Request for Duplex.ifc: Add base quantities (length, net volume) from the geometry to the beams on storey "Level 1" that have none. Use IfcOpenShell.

First a look at what the model holds.

```python
import ifcopenshell
import ifcopenshell.util.element
import ifcopenshell.util.unit

model = ifcopenshell.open("Duplex.ifc")
print(model.schema)
for unit_type in ("LENGTHUNIT", "AREAUNIT", "VOLUMEUNIT"):
    print(unit_type, ifcopenshell.util.unit.calculate_unit_scale(model, unit_type))
storey = next(s for s in model.by_type("IfcBuildingStorey") if s.Name == "Level 1")
beams = [e for e in ifcopenshell.util.element.get_decomposition(storey) if e.is_a("IfcBeam")]
for e in sorted(beams, key=lambda e: e.id()):
    print(e.id(), e.is_a(), e.Name, list(ifcopenshell.util.element.get_psets(e, qtos_only=True)), sep=" | ")
```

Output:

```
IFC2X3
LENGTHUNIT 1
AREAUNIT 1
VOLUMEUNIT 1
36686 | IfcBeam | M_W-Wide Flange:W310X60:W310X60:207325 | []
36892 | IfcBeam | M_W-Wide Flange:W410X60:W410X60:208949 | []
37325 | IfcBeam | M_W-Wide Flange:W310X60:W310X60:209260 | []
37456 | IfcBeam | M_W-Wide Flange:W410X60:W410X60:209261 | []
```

```python
import ifcopenshell
import ifcopenshell.api.pset
import ifcopenshell.geom
import ifcopenshell.util.element
import ifcopenshell.util.shape
import ifcopenshell.util.unit

model = ifcopenshell.open("Duplex.ifc")
unit_scale = ifcopenshell.util.unit.calculate_unit_scale(model)
volume_scale = ifcopenshell.util.unit.calculate_unit_scale(model, "VOLUMEUNIT")
settings = ifcopenshell.geom.settings()

storey = next(s for s in model.by_type("IfcBuildingStorey") if s.Name == "Level 1")
beams = [e for e in ifcopenshell.util.element.get_decomposition(storey) if e.is_a("IfcBeam")]

for e in sorted(beams, key=lambda e: e.id()):
    if ifcopenshell.util.element.get_psets(e, qtos_only=True, should_inherit=False):
        continue
    # Geometry comes back in metres, in the element's own axes.
    shape = ifcopenshell.geom.create_shape(settings, e)
    values = {
        "Length": ifcopenshell.util.shape.get_max_xyz(shape.geometry) / unit_scale,
        "NetVolume": ifcopenshell.util.shape.get_volume(shape.geometry) / volume_scale,
    }
    qto = ifcopenshell.api.pset.add_qto(model, product=e, name="BaseQuantities")
    ifcopenshell.api.pset.edit_qto(model, qto=qto, properties=values)
    print(e.id(), {k: round(v, 3) for k, v in values.items()})

model.write("Duplex_v2.ifc")
```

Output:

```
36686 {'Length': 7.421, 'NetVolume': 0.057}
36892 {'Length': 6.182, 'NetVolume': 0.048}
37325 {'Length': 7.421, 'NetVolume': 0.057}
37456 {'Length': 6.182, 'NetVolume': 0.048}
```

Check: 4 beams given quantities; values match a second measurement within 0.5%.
